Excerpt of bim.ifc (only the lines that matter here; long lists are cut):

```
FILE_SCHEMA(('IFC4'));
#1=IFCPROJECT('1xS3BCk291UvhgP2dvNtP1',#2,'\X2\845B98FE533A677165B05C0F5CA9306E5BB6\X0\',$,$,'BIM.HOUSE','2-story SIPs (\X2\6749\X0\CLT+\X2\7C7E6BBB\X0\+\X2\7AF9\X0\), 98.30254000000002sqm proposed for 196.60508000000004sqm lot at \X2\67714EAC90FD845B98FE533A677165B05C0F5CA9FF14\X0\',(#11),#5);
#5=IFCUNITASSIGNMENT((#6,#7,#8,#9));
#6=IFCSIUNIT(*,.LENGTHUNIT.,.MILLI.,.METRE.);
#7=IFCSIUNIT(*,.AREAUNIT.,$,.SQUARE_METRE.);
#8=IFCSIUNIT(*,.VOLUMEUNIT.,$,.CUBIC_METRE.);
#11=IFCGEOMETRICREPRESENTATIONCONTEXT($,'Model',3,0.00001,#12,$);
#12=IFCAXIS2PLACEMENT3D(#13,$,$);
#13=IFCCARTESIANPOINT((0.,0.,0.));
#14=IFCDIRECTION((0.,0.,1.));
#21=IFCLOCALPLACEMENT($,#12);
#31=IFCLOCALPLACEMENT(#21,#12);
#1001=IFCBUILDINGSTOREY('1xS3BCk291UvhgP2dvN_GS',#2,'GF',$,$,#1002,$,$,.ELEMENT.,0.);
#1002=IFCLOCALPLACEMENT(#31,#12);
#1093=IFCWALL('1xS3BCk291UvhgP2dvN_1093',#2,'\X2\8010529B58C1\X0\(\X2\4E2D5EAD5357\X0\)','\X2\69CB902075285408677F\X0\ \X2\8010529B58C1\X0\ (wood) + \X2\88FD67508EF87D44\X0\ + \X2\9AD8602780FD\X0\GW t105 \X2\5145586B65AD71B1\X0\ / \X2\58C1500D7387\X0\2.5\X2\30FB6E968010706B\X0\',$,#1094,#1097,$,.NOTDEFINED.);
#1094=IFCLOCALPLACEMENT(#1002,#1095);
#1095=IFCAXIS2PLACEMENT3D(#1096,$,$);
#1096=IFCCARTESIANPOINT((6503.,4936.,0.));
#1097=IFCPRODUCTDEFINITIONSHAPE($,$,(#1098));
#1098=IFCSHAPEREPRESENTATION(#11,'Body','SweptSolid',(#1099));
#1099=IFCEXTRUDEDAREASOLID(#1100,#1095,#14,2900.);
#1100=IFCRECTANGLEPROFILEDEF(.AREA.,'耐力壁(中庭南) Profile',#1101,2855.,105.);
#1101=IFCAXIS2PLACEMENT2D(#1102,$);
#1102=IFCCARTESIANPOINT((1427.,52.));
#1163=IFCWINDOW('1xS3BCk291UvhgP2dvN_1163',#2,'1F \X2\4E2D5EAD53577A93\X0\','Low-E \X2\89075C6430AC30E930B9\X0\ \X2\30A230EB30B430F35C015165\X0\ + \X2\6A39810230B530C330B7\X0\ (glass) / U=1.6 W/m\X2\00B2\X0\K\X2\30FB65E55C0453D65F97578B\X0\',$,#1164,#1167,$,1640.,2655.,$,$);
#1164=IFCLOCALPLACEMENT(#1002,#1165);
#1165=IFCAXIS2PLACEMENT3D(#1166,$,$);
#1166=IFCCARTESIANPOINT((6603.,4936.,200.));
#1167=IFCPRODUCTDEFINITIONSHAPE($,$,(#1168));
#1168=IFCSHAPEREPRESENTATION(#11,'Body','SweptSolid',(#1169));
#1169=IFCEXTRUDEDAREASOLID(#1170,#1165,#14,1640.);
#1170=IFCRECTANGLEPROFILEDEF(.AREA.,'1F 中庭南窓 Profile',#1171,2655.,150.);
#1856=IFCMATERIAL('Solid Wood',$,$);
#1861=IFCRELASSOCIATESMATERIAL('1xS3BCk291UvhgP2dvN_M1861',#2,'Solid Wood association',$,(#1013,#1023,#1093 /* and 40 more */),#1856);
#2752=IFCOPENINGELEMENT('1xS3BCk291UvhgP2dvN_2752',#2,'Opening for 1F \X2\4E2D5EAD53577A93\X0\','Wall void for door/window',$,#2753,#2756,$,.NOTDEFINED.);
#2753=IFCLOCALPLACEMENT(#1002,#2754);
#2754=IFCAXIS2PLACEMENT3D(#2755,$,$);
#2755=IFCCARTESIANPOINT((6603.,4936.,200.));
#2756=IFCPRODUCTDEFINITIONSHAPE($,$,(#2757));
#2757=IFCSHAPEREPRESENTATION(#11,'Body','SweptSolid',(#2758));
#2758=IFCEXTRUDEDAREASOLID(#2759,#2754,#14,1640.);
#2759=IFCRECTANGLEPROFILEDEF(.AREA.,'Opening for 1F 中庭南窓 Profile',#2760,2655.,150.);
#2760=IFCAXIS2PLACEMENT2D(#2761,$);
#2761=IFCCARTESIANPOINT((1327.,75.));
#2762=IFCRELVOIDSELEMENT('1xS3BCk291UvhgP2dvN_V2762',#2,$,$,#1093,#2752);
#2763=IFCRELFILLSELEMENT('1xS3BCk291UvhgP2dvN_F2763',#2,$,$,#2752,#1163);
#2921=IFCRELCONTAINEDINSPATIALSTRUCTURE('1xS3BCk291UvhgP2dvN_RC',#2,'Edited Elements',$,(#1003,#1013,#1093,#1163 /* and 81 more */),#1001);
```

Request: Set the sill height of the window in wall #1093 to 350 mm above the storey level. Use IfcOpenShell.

```python
import numpy as np
import ifcopenshell
import ifcopenshell.api.geometry
import ifcopenshell.geom
import ifcopenshell.util.element
import ifcopenshell.util.placement
import ifcopenshell.util.shape
import ifcopenshell.util.unit

model = ifcopenshell.open("bim.ifc")
unit_scale = ifcopenshell.util.unit.calculate_unit_scale(model)

window = model.by_guid("1xS3BCk291UvhgP2dvN_1163")
opening = window.FillsVoids[0].RelatingOpeningElement
storey = ifcopenshell.util.element.get_container(window, ifc_class="IfcBuildingStorey")
level = ifcopenshell.util.placement.get_local_placement(storey.ObjectPlacement)[2, 3]

# The opening's origin need not be at the sill, so measure its lowest point.
shape = ifcopenshell.geom.create_shape(ifcopenshell.geom.settings(), opening)
bottom = ifcopenshell.util.shape.get_shape_bottom_elevation(shape, shape.geometry) / unit_scale
dz = level + 0.35 / unit_scale - bottom

shift = np.array([0.0, 0.0, dz])
# The window is not placed relative to its opening, so move both.
for product in (opening, window):
    matrix = ifcopenshell.util.placement.get_local_placement(product.ObjectPlacement)
    matrix[:3, 3] += shift
    ifcopenshell.api.geometry.edit_object_placement(model, product=product, matrix=matrix, is_si=False)

print(f"moved by {dz * unit_scale:+.3f} m")

model.write("bim_edited.ifc")
```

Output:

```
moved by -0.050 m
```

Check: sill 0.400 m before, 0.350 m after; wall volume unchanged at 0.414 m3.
